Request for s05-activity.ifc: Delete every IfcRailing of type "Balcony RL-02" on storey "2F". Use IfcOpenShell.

First a look at what the model holds.

```python
import ifcopenshell
import ifcopenshell.util.element

model = ifcopenshell.open("s05-activity.ifc")
print(model.schema)
storey = next(s for s in model.by_type("IfcBuildingStorey") if s.Name == "2F")
railings = [e for e in ifcopenshell.util.element.get_decomposition(storey) if e.is_a("IfcRailing")]
seen = {}
for e in railings:
    element_type = ifcopenshell.util.element.get_type(e)
    name = element_type.Name if element_type not in (None, e) else None
    seen[name] = seen.get(name, 0) + 1
for name, count in sorted(seen.items(), key=str):
    print(count, "x", name)
```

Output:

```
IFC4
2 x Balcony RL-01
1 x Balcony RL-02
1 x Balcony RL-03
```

```python
import ifcopenshell
import ifcopenshell.api.root
import ifcopenshell.util.element

model = ifcopenshell.open("s05-activity.ifc")

storey = next(s for s in model.by_type("IfcBuildingStorey") if s.Name == "2F")
railings = [e for e in ifcopenshell.util.element.get_decomposition(storey) if e.is_a("IfcRailing")]
targets = [e for e in railings if (t := ifcopenshell.util.element.get_type(e)) not in (None, e) and t.Name == "Balcony RL-02"]

for e in targets:
    ifcopenshell.api.root.remove_product(model, product=e)
print(len(targets), "removed")

model.write("s05-activity_rev.ifc")
```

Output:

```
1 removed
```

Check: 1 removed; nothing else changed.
